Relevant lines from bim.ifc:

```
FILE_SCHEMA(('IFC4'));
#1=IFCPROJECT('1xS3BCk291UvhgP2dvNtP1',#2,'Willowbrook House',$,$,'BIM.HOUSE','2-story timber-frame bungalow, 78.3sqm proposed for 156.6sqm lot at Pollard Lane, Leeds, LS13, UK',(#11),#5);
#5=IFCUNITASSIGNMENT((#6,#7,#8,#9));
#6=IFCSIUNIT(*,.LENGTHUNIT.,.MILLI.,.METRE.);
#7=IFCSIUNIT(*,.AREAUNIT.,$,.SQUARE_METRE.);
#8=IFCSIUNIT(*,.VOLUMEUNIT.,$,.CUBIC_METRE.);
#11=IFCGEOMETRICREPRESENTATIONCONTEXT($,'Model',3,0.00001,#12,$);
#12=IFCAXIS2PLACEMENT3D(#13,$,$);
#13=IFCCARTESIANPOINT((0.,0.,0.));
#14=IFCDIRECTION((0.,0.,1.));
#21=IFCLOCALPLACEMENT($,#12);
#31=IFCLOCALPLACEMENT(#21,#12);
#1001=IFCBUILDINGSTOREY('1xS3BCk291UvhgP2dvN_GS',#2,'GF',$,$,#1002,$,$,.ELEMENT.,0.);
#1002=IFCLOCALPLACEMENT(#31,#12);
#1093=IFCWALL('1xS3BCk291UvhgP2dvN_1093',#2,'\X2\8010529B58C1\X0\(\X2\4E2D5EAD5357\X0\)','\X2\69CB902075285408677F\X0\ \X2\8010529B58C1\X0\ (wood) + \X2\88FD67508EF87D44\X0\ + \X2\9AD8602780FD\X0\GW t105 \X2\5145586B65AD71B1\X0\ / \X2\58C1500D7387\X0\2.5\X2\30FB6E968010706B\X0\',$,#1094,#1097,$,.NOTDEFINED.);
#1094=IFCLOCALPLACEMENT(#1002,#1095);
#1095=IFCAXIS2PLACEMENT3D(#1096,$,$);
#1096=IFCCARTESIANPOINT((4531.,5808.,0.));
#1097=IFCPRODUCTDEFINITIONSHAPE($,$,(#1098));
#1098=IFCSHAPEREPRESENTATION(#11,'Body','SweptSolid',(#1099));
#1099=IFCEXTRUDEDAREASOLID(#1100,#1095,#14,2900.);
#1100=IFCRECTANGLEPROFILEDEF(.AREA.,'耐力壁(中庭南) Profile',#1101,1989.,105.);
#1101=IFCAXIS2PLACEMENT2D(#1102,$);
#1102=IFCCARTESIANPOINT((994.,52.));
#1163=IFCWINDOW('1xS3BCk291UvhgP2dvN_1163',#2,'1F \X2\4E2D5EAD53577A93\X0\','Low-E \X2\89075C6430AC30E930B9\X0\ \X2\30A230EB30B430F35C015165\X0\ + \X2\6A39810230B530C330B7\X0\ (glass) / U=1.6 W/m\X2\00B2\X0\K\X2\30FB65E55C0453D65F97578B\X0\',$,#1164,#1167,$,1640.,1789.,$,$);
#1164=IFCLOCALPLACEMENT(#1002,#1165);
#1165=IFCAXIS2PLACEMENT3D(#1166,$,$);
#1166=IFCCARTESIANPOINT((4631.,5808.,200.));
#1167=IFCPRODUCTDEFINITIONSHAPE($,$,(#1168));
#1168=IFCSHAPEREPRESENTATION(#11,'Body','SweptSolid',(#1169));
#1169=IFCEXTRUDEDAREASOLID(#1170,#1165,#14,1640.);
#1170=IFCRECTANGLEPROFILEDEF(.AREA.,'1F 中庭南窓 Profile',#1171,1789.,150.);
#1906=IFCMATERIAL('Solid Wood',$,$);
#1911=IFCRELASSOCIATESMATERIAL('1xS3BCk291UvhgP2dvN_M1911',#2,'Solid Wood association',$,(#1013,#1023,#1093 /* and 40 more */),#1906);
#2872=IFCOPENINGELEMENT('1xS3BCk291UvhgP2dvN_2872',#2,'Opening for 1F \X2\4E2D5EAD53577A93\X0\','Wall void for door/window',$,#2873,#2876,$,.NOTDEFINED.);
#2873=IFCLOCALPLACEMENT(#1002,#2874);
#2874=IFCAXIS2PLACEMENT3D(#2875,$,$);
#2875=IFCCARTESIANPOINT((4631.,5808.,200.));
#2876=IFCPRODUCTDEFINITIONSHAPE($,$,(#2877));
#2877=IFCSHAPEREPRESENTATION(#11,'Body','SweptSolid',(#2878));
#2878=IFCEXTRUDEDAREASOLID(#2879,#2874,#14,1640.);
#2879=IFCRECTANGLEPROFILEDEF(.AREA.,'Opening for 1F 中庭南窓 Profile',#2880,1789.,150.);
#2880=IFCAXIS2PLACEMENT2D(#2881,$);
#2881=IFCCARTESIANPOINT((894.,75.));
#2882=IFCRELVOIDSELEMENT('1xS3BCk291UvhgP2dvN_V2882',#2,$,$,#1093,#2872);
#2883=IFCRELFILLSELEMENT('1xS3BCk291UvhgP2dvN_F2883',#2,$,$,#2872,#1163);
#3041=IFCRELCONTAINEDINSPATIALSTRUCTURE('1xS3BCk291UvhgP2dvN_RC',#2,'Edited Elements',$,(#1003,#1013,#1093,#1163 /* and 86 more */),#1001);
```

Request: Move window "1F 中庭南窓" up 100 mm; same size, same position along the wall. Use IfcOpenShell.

```python
import numpy as np
import ifcopenshell
import ifcopenshell.api.geometry
import ifcopenshell.util.placement
import ifcopenshell.util.unit

model = ifcopenshell.open("bim.ifc")
unit_scale = ifcopenshell.util.unit.calculate_unit_scale(model)

window = model.by_guid("1xS3BCk291UvhgP2dvN_1163")
opening = window.FillsVoids[0].RelatingOpeningElement
dz = 0.1 / unit_scale

shift = np.array([0.0, 0.0, dz])
# The window is not placed relative to its opening, so move both.
for product in (opening, window):
    matrix = ifcopenshell.util.placement.get_local_placement(product.ObjectPlacement)
    matrix[:3, 3] += shift
    ifcopenshell.api.geometry.edit_object_placement(model, product=product, matrix=matrix, is_si=False)

print(f"moved by {dz * unit_scale:+.3f} m")

model.write("bim_rev.ifc")
```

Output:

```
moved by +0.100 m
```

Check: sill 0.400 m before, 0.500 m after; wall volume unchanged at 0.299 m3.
